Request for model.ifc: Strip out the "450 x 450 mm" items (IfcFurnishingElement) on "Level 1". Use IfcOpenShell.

First a look at what the model holds.

```python
import ifcopenshell
import ifcopenshell.util.element

model = ifcopenshell.open("model.ifc")
print(model.schema)
storey = next(s for s in model.by_type("IfcBuildingStorey") if s.Name == "Level 1")
furniture = [e for e in ifcopenshell.util.element.get_decomposition(storey) if e.is_a("IfcFurnishingElement")]
seen = {}
for e in furniture:
    element_type = ifcopenshell.util.element.get_type(e)
    name = element_type.Name if element_type not in (None, e) else None
    seen[name] = seen.get(name, 0) + 1
for name, count in sorted(seen.items(), key=str):
    print(count, "x", name)
```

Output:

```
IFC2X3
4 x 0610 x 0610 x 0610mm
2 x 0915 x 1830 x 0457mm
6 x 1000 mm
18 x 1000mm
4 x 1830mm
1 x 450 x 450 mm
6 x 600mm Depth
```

```python
import ifcopenshell
import ifcopenshell.api.root
import ifcopenshell.util.element

model = ifcopenshell.open("model.ifc")

storey = next(s for s in model.by_type("IfcBuildingStorey") if s.Name == "Level 1")
furniture = [e for e in ifcopenshell.util.element.get_decomposition(storey) if e.is_a("IfcFurnishingElement")]
targets = [e for e in furniture if (t := ifcopenshell.util.element.get_type(e)) not in (None, e) and t.Name == "450 x 450 mm"]

for e in targets:
    ifcopenshell.api.root.remove_product(model, product=e)
print(len(targets), "removed")

model.write("model_edited.ifc")
```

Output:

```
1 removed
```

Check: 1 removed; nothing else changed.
